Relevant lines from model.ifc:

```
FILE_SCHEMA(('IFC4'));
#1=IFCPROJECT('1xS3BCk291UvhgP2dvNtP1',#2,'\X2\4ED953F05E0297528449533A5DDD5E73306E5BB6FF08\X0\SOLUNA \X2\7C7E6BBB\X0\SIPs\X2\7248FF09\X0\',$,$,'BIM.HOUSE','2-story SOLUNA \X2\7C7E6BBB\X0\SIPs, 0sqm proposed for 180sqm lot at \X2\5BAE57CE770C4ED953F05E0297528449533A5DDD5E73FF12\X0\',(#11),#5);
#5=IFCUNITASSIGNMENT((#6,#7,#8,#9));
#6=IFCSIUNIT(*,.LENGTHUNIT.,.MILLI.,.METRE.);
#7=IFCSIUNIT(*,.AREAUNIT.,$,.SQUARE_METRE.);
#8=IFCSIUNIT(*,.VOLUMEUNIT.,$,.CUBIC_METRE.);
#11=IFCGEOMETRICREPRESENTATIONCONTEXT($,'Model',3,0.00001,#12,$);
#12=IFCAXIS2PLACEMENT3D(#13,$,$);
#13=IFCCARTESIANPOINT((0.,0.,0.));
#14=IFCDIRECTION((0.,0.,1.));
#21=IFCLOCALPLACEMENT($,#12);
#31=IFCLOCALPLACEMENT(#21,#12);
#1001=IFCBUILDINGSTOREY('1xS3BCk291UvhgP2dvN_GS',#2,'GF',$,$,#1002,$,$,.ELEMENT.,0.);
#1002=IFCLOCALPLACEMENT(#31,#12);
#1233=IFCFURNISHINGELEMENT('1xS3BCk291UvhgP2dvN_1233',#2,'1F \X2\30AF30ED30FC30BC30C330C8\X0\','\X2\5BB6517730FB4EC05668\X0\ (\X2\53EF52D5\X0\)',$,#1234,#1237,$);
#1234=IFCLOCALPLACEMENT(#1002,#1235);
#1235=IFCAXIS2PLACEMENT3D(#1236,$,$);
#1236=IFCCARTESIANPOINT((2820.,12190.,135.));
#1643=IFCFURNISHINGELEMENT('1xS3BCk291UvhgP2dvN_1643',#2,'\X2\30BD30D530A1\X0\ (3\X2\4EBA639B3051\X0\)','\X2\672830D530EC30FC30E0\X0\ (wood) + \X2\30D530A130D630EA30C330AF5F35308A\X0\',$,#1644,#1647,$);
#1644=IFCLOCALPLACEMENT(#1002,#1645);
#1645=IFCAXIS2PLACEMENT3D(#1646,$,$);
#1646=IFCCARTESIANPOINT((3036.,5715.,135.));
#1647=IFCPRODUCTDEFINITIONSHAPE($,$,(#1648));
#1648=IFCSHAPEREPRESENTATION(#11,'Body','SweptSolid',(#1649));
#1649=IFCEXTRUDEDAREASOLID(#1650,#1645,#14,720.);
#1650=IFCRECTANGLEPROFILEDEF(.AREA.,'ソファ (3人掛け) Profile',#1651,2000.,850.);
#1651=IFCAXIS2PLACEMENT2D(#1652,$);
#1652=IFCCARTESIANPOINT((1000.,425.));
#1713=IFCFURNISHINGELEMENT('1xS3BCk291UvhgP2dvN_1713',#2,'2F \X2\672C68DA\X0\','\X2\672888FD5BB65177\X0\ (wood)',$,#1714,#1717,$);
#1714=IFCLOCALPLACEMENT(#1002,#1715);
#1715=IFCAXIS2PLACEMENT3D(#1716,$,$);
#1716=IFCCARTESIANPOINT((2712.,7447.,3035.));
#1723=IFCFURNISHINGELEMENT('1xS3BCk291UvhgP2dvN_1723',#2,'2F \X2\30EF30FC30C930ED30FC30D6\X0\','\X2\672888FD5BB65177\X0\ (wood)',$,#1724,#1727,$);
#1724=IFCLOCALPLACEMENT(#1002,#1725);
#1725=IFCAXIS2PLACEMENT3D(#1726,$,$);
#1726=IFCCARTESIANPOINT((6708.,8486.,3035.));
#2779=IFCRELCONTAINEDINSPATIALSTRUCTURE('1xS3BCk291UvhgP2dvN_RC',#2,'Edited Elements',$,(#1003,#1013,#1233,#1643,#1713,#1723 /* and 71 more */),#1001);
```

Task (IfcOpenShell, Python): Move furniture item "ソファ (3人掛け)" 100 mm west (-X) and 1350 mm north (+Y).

```python
import ifcopenshell
import ifcopenshell.api.geometry
import ifcopenshell.util.placement
import ifcopenshell.util.unit

model = ifcopenshell.open("model.ifc")
unit_scale = ifcopenshell.util.unit.calculate_unit_scale(model)

item = model.by_id(1643)
matrix = ifcopenshell.util.placement.get_local_placement(item.ObjectPlacement)
matrix[0, 3] -= 0.1 / unit_scale
matrix[1, 3] += 1.35 / unit_scale
ifcopenshell.api.geometry.edit_object_placement(model, product=item, matrix=matrix, is_si=False)

print(ifcopenshell.util.placement.get_local_placement(item.ObjectPlacement).round(3) + 0.0)

model.write("model_updated.ifc")
```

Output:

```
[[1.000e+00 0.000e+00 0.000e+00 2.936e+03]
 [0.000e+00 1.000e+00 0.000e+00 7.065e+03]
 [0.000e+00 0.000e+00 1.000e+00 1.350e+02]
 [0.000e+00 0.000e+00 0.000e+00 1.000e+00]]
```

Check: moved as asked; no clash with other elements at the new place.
